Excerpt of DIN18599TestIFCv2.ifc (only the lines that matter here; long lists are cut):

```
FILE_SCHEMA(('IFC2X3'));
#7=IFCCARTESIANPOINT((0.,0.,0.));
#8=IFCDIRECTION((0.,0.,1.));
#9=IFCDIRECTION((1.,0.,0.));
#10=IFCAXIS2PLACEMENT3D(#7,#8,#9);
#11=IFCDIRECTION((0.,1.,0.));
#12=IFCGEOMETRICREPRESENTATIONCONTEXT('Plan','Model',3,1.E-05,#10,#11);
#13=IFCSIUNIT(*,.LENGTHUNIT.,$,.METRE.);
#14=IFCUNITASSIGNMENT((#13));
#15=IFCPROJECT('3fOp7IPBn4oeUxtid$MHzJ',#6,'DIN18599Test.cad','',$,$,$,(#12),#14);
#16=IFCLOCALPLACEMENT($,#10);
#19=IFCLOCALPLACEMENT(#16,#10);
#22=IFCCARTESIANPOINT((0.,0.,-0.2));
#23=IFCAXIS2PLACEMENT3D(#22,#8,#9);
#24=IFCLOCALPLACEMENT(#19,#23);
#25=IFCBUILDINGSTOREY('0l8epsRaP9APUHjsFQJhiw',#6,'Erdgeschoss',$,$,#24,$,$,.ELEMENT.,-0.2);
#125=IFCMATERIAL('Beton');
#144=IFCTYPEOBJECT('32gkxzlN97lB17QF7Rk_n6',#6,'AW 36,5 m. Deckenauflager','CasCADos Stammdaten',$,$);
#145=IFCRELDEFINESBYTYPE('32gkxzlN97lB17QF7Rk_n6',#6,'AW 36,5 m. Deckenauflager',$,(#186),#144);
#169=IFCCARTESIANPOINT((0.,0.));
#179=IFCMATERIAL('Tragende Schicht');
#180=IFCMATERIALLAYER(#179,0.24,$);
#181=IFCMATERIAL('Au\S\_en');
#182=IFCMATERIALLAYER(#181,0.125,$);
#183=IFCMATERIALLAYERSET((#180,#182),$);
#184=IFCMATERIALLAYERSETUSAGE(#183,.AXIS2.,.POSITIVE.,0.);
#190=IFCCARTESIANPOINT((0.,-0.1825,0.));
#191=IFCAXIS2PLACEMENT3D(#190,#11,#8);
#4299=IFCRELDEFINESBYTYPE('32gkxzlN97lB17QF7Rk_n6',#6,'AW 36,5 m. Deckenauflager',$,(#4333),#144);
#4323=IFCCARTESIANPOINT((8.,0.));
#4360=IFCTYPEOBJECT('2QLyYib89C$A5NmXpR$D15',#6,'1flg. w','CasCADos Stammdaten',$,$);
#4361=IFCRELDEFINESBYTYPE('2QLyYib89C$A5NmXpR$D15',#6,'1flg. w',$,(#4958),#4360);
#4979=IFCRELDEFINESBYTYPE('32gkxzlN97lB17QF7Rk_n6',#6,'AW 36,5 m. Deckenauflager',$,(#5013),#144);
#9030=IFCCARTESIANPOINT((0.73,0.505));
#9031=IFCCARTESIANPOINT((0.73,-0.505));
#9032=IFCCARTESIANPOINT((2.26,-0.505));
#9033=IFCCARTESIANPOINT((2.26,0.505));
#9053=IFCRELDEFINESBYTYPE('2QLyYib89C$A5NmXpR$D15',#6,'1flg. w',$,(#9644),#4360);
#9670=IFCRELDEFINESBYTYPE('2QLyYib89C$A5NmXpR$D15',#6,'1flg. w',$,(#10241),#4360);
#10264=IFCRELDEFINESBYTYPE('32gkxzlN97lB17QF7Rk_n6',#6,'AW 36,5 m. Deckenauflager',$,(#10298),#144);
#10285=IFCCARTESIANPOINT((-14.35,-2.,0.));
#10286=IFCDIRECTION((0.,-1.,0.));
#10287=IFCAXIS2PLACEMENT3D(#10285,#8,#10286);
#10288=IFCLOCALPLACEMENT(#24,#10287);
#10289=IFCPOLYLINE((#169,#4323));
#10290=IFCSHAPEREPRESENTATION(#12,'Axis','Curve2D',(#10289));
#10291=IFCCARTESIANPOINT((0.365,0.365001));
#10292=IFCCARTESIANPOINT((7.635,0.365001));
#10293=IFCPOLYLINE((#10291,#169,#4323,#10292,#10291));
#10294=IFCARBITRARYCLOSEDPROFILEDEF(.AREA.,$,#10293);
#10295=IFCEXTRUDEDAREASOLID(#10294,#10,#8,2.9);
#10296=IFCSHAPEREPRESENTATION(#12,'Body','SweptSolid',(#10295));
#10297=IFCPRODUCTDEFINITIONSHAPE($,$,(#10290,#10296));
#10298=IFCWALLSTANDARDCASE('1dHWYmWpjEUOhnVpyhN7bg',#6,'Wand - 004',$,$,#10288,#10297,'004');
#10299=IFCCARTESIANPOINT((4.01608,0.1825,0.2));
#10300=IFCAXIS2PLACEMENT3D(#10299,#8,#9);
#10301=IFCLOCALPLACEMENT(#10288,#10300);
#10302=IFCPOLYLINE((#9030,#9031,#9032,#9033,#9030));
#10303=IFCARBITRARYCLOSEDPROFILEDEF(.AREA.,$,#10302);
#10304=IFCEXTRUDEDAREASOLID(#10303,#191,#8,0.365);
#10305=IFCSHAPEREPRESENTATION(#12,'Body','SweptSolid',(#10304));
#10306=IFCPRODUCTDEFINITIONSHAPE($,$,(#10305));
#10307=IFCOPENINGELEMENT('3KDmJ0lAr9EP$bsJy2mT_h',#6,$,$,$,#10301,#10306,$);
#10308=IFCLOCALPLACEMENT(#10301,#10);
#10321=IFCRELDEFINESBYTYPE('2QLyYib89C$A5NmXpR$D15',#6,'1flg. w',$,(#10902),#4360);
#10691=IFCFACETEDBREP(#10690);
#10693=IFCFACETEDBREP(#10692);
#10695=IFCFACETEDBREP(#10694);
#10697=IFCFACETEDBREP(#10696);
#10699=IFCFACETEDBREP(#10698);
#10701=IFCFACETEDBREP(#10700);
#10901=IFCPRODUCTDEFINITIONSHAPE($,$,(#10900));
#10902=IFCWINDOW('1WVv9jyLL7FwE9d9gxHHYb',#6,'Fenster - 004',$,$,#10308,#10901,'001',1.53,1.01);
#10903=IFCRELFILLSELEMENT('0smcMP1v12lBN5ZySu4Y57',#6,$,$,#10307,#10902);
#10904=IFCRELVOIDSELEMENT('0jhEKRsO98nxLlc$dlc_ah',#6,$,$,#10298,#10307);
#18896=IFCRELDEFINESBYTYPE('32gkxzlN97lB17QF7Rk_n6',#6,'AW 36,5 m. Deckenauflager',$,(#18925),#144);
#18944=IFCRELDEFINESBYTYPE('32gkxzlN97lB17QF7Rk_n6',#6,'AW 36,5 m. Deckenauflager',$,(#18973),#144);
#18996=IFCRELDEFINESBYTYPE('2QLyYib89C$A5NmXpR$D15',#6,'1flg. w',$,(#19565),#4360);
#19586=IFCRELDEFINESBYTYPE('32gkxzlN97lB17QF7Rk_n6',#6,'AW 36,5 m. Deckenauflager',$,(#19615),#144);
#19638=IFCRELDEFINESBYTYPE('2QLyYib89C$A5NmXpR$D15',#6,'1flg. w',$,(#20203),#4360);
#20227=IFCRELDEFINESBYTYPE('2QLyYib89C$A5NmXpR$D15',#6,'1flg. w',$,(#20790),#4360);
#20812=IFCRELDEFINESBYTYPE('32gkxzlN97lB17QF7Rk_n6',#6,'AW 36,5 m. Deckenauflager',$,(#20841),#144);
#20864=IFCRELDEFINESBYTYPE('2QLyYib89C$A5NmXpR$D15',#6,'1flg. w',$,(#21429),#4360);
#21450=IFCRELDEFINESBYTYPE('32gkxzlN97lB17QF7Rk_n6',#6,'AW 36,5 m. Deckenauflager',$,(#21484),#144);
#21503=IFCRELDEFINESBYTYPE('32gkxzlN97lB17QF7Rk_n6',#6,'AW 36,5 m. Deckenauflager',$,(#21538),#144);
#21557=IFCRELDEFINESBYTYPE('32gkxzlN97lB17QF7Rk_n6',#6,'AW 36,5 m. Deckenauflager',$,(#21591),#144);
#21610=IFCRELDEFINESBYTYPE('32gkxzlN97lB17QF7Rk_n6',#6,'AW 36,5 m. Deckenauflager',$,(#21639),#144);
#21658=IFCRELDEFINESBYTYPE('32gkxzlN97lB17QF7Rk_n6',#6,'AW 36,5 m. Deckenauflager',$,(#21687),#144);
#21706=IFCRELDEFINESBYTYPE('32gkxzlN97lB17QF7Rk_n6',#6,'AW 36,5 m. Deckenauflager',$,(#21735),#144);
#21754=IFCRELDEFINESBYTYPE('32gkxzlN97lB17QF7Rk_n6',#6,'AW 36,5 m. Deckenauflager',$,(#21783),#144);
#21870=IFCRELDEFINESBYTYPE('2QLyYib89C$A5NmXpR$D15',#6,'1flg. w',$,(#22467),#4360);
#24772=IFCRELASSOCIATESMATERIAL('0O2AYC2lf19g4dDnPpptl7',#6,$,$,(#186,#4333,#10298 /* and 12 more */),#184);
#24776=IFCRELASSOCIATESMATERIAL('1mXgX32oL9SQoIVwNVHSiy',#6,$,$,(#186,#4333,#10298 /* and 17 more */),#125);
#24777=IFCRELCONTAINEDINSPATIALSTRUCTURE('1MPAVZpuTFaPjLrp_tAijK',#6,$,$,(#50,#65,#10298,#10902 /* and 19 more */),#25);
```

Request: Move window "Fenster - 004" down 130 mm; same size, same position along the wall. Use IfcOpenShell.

```python
import numpy as np
import ifcopenshell
import ifcopenshell.api.geometry
import ifcopenshell.util.placement
import ifcopenshell.util.unit

model = ifcopenshell.open("DIN18599TestIFCv2.ifc")
unit_scale = ifcopenshell.util.unit.calculate_unit_scale(model)

window = model.by_id(10902)
opening = window.FillsVoids[0].RelatingOpeningElement
dz = -0.13

shift = np.array([0.0, 0.0, dz])
# The window is placed relative to its opening, so it follows when the opening moves.
matrix = ifcopenshell.util.placement.get_local_placement(opening.ObjectPlacement)
matrix[:3, 3] += shift
ifcopenshell.api.geometry.edit_object_placement(
    model, product=opening, matrix=matrix, is_si=False, should_transform_children=True
)

print(f"moved by {dz * unit_scale:+.3f} m")

model.write("DIN18599TestIFCv2-out.ifc")
```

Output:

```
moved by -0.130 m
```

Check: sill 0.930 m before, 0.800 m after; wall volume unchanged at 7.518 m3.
